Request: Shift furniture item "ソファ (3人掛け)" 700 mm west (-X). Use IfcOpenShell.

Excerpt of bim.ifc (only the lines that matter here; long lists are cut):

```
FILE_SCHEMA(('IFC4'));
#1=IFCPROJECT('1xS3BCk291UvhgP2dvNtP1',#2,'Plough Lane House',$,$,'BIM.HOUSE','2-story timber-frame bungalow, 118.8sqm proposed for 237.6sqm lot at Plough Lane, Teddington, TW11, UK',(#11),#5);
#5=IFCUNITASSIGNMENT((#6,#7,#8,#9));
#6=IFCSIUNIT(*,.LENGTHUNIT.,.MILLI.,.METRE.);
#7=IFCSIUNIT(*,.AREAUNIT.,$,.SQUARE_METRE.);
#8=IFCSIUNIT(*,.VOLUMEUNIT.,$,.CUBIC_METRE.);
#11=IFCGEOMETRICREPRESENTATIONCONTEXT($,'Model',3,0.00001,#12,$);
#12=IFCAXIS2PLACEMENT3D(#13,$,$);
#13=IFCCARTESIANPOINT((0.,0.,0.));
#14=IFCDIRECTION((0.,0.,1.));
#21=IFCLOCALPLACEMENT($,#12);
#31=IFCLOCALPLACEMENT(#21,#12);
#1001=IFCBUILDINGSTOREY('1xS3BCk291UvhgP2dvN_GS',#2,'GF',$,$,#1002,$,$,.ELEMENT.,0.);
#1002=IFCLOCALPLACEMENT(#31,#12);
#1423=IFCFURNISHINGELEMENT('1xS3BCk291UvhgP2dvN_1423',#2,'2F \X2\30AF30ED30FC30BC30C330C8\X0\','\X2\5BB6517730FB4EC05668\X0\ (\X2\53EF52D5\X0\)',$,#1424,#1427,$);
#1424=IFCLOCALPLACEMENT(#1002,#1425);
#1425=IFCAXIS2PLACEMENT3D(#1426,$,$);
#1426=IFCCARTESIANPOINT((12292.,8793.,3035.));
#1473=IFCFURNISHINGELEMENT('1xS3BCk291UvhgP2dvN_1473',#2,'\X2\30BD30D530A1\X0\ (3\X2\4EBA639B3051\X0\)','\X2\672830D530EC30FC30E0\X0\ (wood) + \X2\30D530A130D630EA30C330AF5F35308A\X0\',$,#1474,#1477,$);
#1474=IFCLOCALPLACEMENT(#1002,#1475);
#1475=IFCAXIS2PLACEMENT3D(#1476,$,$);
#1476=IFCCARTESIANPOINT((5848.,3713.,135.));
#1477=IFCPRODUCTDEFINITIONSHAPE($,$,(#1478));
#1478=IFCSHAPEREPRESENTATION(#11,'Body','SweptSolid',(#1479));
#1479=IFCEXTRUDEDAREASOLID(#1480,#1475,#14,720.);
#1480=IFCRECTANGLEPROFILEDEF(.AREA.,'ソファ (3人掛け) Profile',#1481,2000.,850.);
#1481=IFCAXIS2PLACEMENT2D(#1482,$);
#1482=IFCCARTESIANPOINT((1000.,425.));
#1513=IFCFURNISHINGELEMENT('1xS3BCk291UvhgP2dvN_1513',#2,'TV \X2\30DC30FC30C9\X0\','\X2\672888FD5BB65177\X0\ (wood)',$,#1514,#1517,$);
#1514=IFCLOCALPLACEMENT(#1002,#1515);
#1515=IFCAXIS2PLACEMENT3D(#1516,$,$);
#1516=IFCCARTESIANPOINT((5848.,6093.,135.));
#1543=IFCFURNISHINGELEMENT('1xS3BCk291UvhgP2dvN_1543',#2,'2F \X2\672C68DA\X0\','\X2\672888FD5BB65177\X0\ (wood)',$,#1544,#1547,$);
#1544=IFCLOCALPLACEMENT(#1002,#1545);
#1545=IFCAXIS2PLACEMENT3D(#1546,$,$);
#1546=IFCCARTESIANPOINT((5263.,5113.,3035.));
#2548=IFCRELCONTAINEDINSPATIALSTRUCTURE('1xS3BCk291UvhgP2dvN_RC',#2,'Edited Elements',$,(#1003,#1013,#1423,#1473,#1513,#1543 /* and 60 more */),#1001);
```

```python
import ifcopenshell
import ifcopenshell.api.geometry
import ifcopenshell.util.placement
import ifcopenshell.util.unit

model = ifcopenshell.open("bim.ifc")
unit_scale = ifcopenshell.util.unit.calculate_unit_scale(model)

item = model.by_guid("1xS3BCk291UvhgP2dvN_1473")
matrix = ifcopenshell.util.placement.get_local_placement(item.ObjectPlacement)
matrix[0, 3] -= 0.7 / unit_scale
ifcopenshell.api.geometry.edit_object_placement(model, product=item, matrix=matrix, is_si=False)

print(ifcopenshell.util.placement.get_local_placement(item.ObjectPlacement).round(3) + 0.0)

model.write("bim_edited.ifc")
```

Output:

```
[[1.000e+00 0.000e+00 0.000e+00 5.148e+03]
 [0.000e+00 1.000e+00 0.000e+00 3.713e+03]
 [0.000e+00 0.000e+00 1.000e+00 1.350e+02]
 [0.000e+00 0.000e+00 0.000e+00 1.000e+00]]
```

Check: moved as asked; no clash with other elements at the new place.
